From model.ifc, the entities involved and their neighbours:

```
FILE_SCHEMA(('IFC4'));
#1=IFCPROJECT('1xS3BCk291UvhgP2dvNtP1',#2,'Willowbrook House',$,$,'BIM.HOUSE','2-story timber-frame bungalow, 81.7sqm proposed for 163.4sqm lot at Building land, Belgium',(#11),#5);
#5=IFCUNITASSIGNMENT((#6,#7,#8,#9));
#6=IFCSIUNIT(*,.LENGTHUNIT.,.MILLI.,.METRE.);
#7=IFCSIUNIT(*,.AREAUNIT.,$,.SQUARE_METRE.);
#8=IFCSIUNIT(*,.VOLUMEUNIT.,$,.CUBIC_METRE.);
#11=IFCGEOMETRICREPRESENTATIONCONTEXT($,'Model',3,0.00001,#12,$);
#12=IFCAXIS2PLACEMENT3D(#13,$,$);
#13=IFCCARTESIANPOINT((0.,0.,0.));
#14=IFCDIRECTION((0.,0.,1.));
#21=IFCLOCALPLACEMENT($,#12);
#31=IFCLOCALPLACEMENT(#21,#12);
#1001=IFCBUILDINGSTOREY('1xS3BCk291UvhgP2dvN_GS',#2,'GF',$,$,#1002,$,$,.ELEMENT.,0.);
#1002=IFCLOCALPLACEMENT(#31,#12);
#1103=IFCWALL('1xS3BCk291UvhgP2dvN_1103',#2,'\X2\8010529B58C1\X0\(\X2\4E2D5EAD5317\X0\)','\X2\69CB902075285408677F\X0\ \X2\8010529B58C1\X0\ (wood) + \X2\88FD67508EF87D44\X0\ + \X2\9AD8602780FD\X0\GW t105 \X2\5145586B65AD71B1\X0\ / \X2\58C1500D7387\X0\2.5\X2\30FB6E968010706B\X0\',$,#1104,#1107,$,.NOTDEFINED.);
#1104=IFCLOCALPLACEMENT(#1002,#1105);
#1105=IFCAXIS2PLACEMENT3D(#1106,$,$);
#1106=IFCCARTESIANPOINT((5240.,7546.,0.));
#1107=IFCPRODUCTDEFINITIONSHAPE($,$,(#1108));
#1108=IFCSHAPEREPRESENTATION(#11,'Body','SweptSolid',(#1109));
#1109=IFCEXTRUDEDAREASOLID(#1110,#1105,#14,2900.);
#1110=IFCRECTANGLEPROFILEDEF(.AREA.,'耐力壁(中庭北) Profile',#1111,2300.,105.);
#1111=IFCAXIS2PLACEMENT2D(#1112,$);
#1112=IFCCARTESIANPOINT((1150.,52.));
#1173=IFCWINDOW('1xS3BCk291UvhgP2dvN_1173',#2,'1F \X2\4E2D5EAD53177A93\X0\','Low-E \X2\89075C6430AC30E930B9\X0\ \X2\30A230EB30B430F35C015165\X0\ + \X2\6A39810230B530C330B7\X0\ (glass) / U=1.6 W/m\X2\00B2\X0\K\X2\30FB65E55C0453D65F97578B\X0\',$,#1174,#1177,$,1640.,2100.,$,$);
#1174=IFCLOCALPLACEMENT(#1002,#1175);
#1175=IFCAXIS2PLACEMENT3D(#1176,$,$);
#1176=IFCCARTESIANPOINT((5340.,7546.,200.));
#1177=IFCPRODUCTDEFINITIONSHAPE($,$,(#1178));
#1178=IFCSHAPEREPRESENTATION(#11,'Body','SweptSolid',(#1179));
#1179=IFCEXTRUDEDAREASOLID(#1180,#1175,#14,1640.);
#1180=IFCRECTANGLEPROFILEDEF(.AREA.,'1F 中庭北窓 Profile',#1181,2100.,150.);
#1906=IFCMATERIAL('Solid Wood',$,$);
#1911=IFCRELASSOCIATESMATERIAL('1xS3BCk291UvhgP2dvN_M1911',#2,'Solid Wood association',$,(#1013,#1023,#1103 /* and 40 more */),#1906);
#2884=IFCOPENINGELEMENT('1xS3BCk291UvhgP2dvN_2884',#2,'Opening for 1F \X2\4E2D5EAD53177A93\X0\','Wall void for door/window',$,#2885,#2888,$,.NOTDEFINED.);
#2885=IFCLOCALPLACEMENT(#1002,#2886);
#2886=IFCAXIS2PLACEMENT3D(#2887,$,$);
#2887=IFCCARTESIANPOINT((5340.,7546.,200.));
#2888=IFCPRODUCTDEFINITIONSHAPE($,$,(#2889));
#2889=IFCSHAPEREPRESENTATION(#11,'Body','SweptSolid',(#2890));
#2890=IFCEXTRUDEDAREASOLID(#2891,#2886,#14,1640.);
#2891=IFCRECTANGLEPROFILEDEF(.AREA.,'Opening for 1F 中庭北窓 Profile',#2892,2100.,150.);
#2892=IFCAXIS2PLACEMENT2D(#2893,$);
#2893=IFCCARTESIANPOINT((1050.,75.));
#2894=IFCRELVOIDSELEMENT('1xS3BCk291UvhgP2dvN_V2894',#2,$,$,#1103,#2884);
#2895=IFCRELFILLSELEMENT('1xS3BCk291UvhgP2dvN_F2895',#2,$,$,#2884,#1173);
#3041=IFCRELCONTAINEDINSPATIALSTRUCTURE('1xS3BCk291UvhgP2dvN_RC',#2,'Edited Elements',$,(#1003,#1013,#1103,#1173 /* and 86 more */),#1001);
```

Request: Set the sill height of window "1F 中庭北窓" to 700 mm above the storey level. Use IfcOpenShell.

```python
import numpy as np
import ifcopenshell
import ifcopenshell.api.geometry
import ifcopenshell.geom
import ifcopenshell.util.element
import ifcopenshell.util.placement
import ifcopenshell.util.shape
import ifcopenshell.util.unit

model = ifcopenshell.open("model.ifc")
unit_scale = ifcopenshell.util.unit.calculate_unit_scale(model)

window = model.by_guid("1xS3BCk291UvhgP2dvN_1173")
opening = window.FillsVoids[0].RelatingOpeningElement
storey = ifcopenshell.util.element.get_container(window, ifc_class="IfcBuildingStorey")
level = ifcopenshell.util.placement.get_local_placement(storey.ObjectPlacement)[2, 3]

# The opening's origin need not be at the sill, so measure its lowest point.
shape = ifcopenshell.geom.create_shape(ifcopenshell.geom.settings(), opening)
bottom = ifcopenshell.util.shape.get_shape_bottom_elevation(shape, shape.geometry) / unit_scale
dz = level + 0.7 / unit_scale - bottom

shift = np.array([0.0, 0.0, dz])
# The window is not placed relative to its opening, so move both.
for product in (opening, window):
    matrix = ifcopenshell.util.placement.get_local_placement(product.ObjectPlacement)
    matrix[:3, 3] += shift
    ifcopenshell.api.geometry.edit_object_placement(model, product=product, matrix=matrix, is_si=False)

print(f"moved by {dz * unit_scale:+.3f} m")

model.write("model-out.ifc")
```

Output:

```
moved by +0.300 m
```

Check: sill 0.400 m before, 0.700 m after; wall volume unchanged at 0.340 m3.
